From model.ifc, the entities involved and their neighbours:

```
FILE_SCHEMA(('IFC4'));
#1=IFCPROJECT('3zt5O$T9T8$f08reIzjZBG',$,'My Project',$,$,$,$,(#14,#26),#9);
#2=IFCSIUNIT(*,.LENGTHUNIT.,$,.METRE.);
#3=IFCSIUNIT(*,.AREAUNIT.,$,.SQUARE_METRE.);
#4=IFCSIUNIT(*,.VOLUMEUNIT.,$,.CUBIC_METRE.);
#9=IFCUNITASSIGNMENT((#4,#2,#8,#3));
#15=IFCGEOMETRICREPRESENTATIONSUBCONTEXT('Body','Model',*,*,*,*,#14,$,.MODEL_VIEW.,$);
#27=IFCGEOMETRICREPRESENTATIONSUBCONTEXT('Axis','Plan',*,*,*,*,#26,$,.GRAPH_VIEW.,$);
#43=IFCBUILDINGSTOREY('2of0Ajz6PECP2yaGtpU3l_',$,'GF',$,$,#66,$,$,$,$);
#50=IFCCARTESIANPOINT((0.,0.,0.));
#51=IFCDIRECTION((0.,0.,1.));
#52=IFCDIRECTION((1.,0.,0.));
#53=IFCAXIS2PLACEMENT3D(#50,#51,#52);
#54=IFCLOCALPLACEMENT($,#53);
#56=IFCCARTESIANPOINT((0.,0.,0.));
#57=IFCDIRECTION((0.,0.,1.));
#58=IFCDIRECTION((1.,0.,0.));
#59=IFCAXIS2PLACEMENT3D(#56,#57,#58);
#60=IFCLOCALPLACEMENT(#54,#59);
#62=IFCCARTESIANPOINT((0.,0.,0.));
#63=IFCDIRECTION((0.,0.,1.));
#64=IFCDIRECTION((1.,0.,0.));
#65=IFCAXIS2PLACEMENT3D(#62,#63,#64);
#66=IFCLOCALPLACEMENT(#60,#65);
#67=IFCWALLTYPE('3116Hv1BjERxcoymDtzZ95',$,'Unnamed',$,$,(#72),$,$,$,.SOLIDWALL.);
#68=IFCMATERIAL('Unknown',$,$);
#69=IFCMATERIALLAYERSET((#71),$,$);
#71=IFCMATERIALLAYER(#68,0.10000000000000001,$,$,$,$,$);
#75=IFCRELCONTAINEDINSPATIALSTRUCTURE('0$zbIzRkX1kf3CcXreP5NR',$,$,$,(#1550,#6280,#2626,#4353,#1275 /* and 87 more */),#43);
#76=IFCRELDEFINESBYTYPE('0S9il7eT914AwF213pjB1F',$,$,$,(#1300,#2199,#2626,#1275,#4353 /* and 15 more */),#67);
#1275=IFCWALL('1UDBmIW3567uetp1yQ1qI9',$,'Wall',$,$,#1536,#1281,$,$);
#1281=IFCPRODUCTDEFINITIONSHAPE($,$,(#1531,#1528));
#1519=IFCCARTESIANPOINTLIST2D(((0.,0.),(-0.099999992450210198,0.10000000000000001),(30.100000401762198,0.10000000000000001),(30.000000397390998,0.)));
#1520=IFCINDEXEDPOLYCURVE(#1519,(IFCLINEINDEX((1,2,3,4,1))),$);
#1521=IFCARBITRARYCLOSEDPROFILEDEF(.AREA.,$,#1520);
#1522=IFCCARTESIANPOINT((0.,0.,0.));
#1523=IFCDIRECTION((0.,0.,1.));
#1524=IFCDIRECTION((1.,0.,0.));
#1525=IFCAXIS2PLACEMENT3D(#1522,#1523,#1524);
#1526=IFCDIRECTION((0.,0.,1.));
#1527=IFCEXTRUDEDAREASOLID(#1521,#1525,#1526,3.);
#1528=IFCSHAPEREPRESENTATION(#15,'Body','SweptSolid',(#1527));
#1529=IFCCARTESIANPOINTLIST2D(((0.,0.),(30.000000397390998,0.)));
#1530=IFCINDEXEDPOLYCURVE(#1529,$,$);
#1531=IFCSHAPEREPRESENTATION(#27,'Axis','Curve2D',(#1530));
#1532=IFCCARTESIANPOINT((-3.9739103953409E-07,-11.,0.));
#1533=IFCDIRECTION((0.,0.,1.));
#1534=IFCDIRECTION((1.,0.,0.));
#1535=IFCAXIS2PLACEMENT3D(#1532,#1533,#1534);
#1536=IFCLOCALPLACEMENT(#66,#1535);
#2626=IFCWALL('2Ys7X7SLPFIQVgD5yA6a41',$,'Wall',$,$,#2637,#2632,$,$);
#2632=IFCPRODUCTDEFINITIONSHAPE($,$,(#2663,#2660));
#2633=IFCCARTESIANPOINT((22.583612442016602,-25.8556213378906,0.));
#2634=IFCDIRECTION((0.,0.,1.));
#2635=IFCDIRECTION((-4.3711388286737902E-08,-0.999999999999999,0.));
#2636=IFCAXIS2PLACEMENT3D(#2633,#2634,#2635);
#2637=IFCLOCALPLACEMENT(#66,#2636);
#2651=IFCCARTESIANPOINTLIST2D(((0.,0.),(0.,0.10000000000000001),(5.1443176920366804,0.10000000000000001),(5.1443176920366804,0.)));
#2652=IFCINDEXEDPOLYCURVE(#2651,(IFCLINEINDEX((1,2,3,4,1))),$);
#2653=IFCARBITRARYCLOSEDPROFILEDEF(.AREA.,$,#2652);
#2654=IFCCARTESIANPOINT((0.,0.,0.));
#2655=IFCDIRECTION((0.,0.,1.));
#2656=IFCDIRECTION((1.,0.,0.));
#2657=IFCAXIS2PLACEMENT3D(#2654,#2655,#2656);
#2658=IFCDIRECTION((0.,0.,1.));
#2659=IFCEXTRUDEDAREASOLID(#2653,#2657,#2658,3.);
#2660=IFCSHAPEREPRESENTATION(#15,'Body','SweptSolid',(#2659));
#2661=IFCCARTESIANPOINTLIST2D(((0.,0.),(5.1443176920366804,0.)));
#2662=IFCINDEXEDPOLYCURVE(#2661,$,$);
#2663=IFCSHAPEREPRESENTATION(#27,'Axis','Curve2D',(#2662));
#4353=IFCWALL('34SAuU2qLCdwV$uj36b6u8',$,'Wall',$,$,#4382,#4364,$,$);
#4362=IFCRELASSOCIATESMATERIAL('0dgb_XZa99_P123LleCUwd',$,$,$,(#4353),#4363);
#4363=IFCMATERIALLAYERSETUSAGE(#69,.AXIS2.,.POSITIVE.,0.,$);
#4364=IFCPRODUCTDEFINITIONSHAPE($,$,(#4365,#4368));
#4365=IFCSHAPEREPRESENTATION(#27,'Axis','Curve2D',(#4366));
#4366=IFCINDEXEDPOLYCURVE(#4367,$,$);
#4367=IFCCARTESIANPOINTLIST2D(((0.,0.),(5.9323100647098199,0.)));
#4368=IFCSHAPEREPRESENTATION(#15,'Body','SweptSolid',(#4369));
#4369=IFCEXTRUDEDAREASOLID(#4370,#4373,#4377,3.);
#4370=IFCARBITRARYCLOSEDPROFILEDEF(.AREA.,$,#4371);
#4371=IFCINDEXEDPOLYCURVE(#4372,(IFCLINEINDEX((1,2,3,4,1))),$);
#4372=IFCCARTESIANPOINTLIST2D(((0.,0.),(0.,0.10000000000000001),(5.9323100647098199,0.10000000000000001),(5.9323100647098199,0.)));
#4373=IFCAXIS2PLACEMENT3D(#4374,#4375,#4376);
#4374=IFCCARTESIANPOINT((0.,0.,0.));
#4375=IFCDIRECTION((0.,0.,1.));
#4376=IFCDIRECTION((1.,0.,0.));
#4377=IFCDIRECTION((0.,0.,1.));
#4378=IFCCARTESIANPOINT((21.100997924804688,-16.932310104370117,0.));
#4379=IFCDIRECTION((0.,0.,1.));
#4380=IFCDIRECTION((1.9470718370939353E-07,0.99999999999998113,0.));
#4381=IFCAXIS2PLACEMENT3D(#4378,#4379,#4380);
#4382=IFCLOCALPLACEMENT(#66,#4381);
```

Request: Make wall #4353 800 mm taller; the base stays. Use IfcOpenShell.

```python
import ifcopenshell
import ifcopenshell.geom
import ifcopenshell.util.representation
import ifcopenshell.util.shape
import ifcopenshell.util.unit

model = ifcopenshell.open("model.ifc")
unit_scale = ifcopenshell.util.unit.calculate_unit_scale(model)
settings = ifcopenshell.geom.settings()


def volume(element):
    """Net volume in cubic metres, openings subtracted."""
    shape = ifcopenshell.geom.create_shape(settings, element)
    return ifcopenshell.util.shape.get_volume(shape.geometry)


wall = model.by_guid("34SAuU2qLCdwV$uj36b6u8")
before = volume(wall)

body = ifcopenshell.util.representation.get_representation(wall, "Model", "Body")
solid = body.Items[0]
old_height = solid.Depth
solid.Depth += 0.8 / unit_scale
after = volume(wall)

print(f"height {old_height:g} -> {solid.Depth:g}, volume {before:.3f} -> {after:.3f} m3")

model.write("model_edited.ifc")
```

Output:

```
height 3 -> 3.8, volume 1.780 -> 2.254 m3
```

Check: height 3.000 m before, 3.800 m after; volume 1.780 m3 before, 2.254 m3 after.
